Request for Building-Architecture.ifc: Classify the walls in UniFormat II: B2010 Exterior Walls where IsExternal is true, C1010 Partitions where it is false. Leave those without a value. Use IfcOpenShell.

First a look at what the model holds.

```python
import ifcopenshell
import ifcopenshell.util.element

model = ifcopenshell.open("Building-Architecture.ifc")
print(model.schema)
print("classifications:", [c.Name for c in model.by_type("IfcClassification")])
values = [ifcopenshell.util.element.get_pset(e, "Pset_WallCommon", "IsExternal") for e in model.by_type("IfcWall")]
for value in (True, False, None):
    print("IsExternal", value, values.count(value))
```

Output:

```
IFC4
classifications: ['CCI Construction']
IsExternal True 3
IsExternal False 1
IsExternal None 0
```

```python
import ifcopenshell
import ifcopenshell.api.classification
import ifcopenshell.util.element

model = ifcopenshell.open("Building-Architecture.ifc")

system = ifcopenshell.api.classification.add_classification(model, classification="UniFormat II")

walls = model.by_type("IfcWall")
external = {e: ifcopenshell.util.element.get_pset(e, "Pset_WallCommon", "IsExternal") for e in walls}
for flag, code, name in ((True, "B2010", "Exterior Walls"), (False, "C1010", "Partitions")):
    products = [e for e in walls if external[e] is flag]
    ifcopenshell.api.classification.add_reference(
        model, products=products, classification=system, identification=code, name=name
    )
    print(code, len(products))

model.write("Building-Architecture_edited.ifc")
```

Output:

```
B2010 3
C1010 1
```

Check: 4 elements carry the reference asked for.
